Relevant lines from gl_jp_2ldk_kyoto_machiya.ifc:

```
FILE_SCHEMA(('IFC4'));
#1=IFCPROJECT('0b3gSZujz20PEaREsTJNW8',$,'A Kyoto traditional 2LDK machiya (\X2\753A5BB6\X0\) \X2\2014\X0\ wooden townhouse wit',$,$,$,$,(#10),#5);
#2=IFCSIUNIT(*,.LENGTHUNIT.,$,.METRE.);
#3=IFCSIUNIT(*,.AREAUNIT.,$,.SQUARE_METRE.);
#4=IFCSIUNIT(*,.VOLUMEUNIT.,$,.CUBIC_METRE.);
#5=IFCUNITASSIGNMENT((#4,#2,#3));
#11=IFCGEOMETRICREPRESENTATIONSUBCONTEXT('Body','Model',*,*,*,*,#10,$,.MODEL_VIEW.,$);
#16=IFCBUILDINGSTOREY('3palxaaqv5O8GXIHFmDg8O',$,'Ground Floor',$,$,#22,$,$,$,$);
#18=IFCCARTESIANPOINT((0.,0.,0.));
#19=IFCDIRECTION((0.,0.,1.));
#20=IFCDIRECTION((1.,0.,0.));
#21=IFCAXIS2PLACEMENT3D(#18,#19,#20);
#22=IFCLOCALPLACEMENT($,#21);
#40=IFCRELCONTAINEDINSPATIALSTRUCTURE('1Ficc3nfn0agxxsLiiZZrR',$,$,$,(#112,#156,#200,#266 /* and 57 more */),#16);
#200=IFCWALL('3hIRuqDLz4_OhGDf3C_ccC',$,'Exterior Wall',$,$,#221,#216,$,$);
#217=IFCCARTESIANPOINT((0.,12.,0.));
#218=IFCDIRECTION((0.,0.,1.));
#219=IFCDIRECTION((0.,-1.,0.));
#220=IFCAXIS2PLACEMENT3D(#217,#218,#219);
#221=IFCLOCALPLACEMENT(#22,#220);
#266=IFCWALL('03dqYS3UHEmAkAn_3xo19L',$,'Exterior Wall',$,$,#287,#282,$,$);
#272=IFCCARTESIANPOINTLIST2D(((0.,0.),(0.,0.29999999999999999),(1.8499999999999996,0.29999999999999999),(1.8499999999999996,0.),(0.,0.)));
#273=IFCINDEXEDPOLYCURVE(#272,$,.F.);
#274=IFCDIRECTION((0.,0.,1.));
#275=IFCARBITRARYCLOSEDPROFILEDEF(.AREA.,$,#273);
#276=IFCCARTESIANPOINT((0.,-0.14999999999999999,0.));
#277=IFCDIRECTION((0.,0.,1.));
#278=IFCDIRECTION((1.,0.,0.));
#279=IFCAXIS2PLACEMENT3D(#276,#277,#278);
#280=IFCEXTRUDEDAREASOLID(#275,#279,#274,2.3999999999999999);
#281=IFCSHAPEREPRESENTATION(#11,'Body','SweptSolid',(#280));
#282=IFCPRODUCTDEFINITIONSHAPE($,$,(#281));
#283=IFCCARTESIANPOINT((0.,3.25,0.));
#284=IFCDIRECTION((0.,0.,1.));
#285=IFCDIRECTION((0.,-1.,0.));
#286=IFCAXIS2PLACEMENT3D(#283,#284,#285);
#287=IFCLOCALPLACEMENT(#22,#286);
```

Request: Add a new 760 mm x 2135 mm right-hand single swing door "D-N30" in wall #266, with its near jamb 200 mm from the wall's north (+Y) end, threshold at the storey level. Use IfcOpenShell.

```python
import numpy as np
import ifcopenshell
import ifcopenshell.api.feature
import ifcopenshell.api.geometry
import ifcopenshell.api.root
import ifcopenshell.api.spatial
import ifcopenshell.geom
import ifcopenshell.util.element
import ifcopenshell.util.placement
import ifcopenshell.util.representation
import ifcopenshell.util.shape
import ifcopenshell.util.unit

model = ifcopenshell.open("gl_jp_2ldk_kyoto_machiya.ifc")
unit_scale = ifcopenshell.util.unit.calculate_unit_scale(model)
settings = ifcopenshell.geom.settings()


def volume(element):
    """Net volume in cubic metres, openings subtracted."""
    shape = ifcopenshell.geom.create_shape(settings, element)
    return ifcopenshell.util.shape.get_volume(shape.geometry)


wall = model.by_guid("03dqYS3UHEmAkAn_3xo19L")
storey = ifcopenshell.util.element.get_container(wall, ifc_class="IfcBuildingStorey")
context = ifcopenshell.util.representation.get_context(model, "Model", "Body", "MODEL_VIEW")
before = volume(wall)

width, height, from_end, sill = 0.76, 2.135, 0.2, 0.0  # metres

# The wall runs along its own X axis, and the end named is its -X end.
wall_shape = ifcopenshell.geom.create_shape(settings, wall)
x, y, z = ifcopenshell.util.shape.get_vertices(wall_shape.geometry).T
start = x.min() + from_end
face, thickness = float(y.min()), float(y.max() - y.min())
wall_matrix = ifcopenshell.util.placement.get_local_placement(wall.ObjectPlacement)
level = ifcopenshell.util.placement.get_local_placement(storey.ObjectPlacement)[2, 3]


def in_wall(x, y):
    """Placement at x, y metres in the wall's axes, at sill height."""
    matrix = wall_matrix.copy()
    matrix[:, 3] = wall_matrix @ np.array([x / unit_scale, y / unit_scale, 0.0, 1.0])
    matrix[2, 3] = level + sill / unit_scale
    return matrix


# Opening: a box that overshoots both wall faces by 50 mm.
opening = ifcopenshell.api.root.create_entity(model, ifc_class="IfcOpeningElement", predefined_type="OPENING")
box = ifcopenshell.api.geometry.add_wall_representation(
    model, context=context, length=width, height=height, thickness=thickness + 0.1
)
ifcopenshell.api.geometry.assign_representation(model, product=opening, representation=box)
ifcopenshell.api.geometry.edit_object_placement(model, product=opening, matrix=in_wall(start, face - 0.05), is_si=False)
ifcopenshell.api.feature.add_feature(model, feature=opening, element=wall)

door = ifcopenshell.api.root.create_entity(model, ifc_class="IfcDoor", name="D-N30", predefined_type="DOOR")
door.OverallWidth, door.OverallHeight = width / unit_scale, height / unit_scale
door.OperationType = "SINGLE_SWING_RIGHT"
body = ifcopenshell.api.geometry.add_door_representation(
    model,
    context=context,
    overall_width=door.OverallWidth,
    overall_height=door.OverallHeight,
    operation_type="SINGLE_SWING_RIGHT",
    lining_properties={"LiningDepth": thickness / unit_scale, "ThresholdDepth": thickness / unit_scale},
)
ifcopenshell.api.geometry.assign_representation(model, product=door, representation=body)
ifcopenshell.api.spatial.assign_container(model, products=[door], relating_structure=storey)
ifcopenshell.api.feature.add_filling(model, opening=opening, element=door)

# The lining spans the wall, so the door starts at the wall face.
ifcopenshell.api.geometry.edit_object_placement(model, product=door, matrix=in_wall(start, face), is_si=False)

after = volume(wall)

print(f"wall volume {before:.3f} -> {after:.3f} m3")

model.write("gl_jp_2ldk_kyoto_machiya_v2.ifc")
```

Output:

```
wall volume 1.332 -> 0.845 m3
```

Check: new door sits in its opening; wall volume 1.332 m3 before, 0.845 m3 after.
